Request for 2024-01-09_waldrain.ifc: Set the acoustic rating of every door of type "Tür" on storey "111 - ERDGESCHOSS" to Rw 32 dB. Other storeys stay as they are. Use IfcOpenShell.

First a look at what the model holds.

```python
import ifcopenshell
import ifcopenshell.util.element

model = ifcopenshell.open("2024-01-09_waldrain.ifc")
print(model.schema)
storey = next(s for s in model.by_type("IfcBuildingStorey") if s.Name == "111 - ERDGESCHOSS")
doors = [e for e in ifcopenshell.util.element.get_decomposition(storey) if e.is_a("IfcDoor")]
seen = {}
for e in doors:
    element_type = ifcopenshell.util.element.get_type(e)
    key = (element_type.Name if element_type != e and element_type else None, ifcopenshell.util.element.get_pset(e, "Pset_DoorCommon", "AcousticRating"))
    seen[key] = seen.get(key, 0) + 1
for (name, value), count in sorted(seen.items(), key=str):
    print(count, "x", name, "|", value)
```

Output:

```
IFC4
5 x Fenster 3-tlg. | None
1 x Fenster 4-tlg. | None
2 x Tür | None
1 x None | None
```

```python
import ifcopenshell
import ifcopenshell.api.pset
import ifcopenshell.util.element

model = ifcopenshell.open("2024-01-09_waldrain.ifc")

storey = next(s for s in model.by_type("IfcBuildingStorey") if s.Name == "111 - ERDGESCHOSS")
doors = [e for e in ifcopenshell.util.element.get_decomposition(storey) if e.is_a("IfcDoor")]

count = 0
for e in doors:
    element_type = ifcopenshell.util.element.get_type(e)
    if element_type in (None, e) or element_type.Name != "Tür":
        continue
    # add_pset returns the element's existing set when there is one.
    pset = ifcopenshell.api.pset.add_pset(model, product=e, name="Pset_DoorCommon")
    ifcopenshell.api.pset.edit_pset(model, pset=pset, properties={"AcousticRating": "Rw 32 dB"})
    count += 1

print(count, "doors updated")

model.write("2024-01-09_waldrain_edited.ifc")
```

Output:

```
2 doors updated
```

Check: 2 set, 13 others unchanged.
